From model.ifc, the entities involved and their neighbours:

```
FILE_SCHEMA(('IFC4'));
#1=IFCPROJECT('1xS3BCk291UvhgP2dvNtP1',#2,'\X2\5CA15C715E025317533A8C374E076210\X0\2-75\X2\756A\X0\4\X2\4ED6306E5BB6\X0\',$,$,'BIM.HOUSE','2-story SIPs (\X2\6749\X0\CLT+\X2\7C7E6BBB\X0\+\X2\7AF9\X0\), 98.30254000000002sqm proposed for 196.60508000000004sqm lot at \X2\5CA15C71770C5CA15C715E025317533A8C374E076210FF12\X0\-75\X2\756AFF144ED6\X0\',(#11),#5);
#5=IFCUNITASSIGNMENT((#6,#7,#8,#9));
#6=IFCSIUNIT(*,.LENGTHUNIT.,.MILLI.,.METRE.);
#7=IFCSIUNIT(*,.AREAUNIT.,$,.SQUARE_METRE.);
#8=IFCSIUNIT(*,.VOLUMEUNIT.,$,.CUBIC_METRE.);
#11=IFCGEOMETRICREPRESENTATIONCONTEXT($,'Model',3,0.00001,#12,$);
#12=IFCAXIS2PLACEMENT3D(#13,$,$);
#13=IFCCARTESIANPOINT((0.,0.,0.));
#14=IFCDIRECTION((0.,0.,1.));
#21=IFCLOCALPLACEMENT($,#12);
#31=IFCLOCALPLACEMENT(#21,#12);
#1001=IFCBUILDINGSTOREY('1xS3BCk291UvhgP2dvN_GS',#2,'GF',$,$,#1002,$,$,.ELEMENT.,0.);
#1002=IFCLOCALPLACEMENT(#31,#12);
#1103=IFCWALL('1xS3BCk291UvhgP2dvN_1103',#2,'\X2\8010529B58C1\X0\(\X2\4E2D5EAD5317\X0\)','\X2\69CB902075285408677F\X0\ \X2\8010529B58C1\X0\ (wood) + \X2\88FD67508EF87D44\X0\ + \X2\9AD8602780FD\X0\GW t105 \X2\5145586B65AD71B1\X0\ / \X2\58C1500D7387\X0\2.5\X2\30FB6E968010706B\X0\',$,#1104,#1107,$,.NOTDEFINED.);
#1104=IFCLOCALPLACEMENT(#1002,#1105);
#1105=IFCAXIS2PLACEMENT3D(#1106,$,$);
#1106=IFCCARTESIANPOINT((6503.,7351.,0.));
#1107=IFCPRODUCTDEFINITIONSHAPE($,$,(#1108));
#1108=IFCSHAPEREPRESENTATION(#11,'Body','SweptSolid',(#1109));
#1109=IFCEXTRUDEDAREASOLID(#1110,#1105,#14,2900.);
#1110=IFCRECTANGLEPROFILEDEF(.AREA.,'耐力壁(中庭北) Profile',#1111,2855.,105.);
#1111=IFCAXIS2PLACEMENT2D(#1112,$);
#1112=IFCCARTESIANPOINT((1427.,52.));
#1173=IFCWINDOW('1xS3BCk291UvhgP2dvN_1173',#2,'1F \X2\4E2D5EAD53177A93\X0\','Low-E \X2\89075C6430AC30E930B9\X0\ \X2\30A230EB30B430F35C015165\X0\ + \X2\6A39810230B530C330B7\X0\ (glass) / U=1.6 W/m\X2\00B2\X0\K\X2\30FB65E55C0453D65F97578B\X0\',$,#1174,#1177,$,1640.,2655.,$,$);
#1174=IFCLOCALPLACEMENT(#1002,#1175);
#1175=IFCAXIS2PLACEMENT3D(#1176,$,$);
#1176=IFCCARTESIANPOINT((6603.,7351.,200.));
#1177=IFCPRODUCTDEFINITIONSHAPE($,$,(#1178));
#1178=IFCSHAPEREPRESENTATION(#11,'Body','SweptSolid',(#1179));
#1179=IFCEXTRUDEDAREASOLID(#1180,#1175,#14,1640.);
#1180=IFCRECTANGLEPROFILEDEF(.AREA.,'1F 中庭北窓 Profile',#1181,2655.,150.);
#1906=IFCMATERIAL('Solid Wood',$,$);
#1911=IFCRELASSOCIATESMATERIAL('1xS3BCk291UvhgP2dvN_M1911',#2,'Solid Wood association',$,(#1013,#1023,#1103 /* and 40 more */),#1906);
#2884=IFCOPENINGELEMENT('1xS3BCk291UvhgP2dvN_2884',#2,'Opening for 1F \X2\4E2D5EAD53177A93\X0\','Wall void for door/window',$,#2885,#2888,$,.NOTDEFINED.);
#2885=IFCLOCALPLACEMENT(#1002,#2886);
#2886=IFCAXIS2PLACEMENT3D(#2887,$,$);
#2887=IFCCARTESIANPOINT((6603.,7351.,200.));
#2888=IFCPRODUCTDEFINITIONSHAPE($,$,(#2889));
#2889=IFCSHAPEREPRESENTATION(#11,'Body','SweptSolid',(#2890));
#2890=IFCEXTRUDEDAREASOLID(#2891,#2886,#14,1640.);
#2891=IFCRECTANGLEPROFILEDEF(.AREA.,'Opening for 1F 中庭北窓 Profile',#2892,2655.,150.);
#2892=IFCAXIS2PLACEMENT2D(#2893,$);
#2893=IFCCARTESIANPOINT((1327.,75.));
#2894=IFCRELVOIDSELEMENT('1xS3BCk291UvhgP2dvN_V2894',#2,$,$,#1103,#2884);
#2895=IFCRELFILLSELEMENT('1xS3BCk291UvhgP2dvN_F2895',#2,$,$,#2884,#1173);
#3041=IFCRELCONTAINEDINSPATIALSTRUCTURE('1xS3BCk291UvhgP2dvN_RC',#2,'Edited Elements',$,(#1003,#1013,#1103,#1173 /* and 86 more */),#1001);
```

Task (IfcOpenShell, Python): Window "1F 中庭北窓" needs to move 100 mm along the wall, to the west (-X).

```python
import ifcopenshell
import ifcopenshell.api.geometry
import ifcopenshell.util.placement
import ifcopenshell.util.unit

model = ifcopenshell.open("model.ifc")
unit_scale = ifcopenshell.util.unit.calculate_unit_scale(model)

window = model.by_id(1173)
opening = window.FillsVoids[0].RelatingOpeningElement
wall = opening.VoidsElements[0].RelatingBuildingElement

wall_matrix = ifcopenshell.util.placement.get_local_placement(wall.ObjectPlacement)
shift = wall_matrix[:3, 0] * -0.1 / unit_scale
before = ifcopenshell.util.placement.get_local_placement(window.ObjectPlacement)[:3, 3].copy()

# The window is not placed relative to its opening, so move both.
for product in (opening, window):
    matrix = ifcopenshell.util.placement.get_local_placement(product.ObjectPlacement)
    matrix[:3, 3] += shift
    ifcopenshell.api.geometry.edit_object_placement(model, product=product, matrix=matrix, is_si=False)

after = ifcopenshell.util.placement.get_local_placement(window.ObjectPlacement)[:3, 3]
print("window moved by", (after - before).round(3) + 0.0)

model.write("model_edited.ifc")
```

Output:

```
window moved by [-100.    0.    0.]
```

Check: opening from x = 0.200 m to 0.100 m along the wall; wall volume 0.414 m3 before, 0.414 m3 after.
